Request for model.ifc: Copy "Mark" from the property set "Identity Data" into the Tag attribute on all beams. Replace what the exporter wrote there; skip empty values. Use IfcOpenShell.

First a look at what the model holds.

```python
import ifcopenshell
import ifcopenshell.util.element

model = ifcopenshell.open("model.ifc")
print(model.schema)
beams = model.by_type("IfcBeam")
print(len(beams), "beams")
for e in beams[:8]:
    source = ifcopenshell.util.element.get_pset(e, "Identity Data", "Mark")
    target = e.Tag
    print(e.id(), repr(source), repr(target), sep=" | ")
```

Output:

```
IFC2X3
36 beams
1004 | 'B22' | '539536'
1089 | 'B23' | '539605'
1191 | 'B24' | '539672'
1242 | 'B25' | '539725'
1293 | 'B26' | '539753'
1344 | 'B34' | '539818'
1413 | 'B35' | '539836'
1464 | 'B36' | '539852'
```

```python
import ifcopenshell
import ifcopenshell.util.element

model = ifcopenshell.open("model.ifc")

count = 0
for e in model.by_type("IfcBeam"):
    value = ifcopenshell.util.element.get_pset(e, "Identity Data", "Mark")
    current = e.Tag
    if not value or not value.strip() or current == value:
        continue
    e.Tag = value
    count += 1

print(count, "beams updated")

model.write("model_updated.ifc")
```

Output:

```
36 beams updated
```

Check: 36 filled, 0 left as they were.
